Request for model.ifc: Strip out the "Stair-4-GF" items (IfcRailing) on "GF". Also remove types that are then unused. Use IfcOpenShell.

First a look at what the model holds.

```python
import ifcopenshell
import ifcopenshell.util.element

model = ifcopenshell.open("model.ifc")
print(model.schema)
storey = next(s for s in model.by_type("IfcBuildingStorey") if s.Name == "GF")
railings = [e for e in ifcopenshell.util.element.get_decomposition(storey) if e.is_a("IfcRailing")]
seen = {}
for e in railings:
    element_type = ifcopenshell.util.element.get_type(e)
    name = element_type.Name if element_type not in (None, e) else None
    seen[name] = seen.get(name, 0) + 1
for name, count in sorted(seen.items(), key=str):
    print(count, "x", name)
```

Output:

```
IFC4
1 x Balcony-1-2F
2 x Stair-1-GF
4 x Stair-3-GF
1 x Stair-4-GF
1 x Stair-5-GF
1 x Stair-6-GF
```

```python
import ifcopenshell
import ifcopenshell.api.root
import ifcopenshell.util.element

model = ifcopenshell.open("model.ifc")

storey = next(s for s in model.by_type("IfcBuildingStorey") if s.Name == "GF")
railings = [e for e in ifcopenshell.util.element.get_decomposition(storey) if e.is_a("IfcRailing")]
targets = [e for e in railings if (t := ifcopenshell.util.element.get_type(e)) not in (None, e) and t.Name == "Stair-4-GF"]
types = {ifcopenshell.util.element.get_type(e) for e in targets} - {None, *targets}

for e in targets:
    ifcopenshell.api.root.remove_product(model, product=e)
print(len(targets), "removed")

unused = [t for t in types if not ifcopenshell.util.element.get_types(t)]
for t in unused:
    ifcopenshell.api.root.remove_product(model, product=t)
print(len(unused), "unused types removed")

model.write("model-out.ifc")
```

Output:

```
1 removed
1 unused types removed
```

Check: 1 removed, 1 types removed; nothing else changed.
